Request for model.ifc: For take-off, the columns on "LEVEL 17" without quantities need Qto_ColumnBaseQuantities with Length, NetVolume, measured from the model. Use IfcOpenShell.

First a look at what the model holds.

```python
import ifcopenshell
import ifcopenshell.util.element
import ifcopenshell.util.unit

model = ifcopenshell.open("model.ifc")
print(model.schema)
for unit_type in ("LENGTHUNIT", "AREAUNIT", "VOLUMEUNIT"):
    print(unit_type, ifcopenshell.util.unit.calculate_unit_scale(model, unit_type))
storey = next(s for s in model.by_type("IfcBuildingStorey") if s.Name == "LEVEL 17")
columns = [e for e in ifcopenshell.util.element.get_decomposition(storey) if e.is_a("IfcColumn")]
for e in sorted(columns, key=lambda e: e.id()):
    print(e.id(), e.is_a(), e.Name, list(ifcopenshell.util.element.get_psets(e, qtos_only=True)), sep=" | ")
```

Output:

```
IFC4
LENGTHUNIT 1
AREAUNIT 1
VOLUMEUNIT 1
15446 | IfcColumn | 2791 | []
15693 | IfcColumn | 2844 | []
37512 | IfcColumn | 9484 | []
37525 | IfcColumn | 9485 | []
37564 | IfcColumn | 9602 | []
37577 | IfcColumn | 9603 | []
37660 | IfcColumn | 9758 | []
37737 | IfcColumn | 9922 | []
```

```python
import ifcopenshell
import ifcopenshell.api.pset
import ifcopenshell.geom
import ifcopenshell.util.element
import ifcopenshell.util.shape
import ifcopenshell.util.unit

model = ifcopenshell.open("model.ifc")
unit_scale = ifcopenshell.util.unit.calculate_unit_scale(model)
volume_scale = ifcopenshell.util.unit.calculate_unit_scale(model, "VOLUMEUNIT")
settings = ifcopenshell.geom.settings()

storey = next(s for s in model.by_type("IfcBuildingStorey") if s.Name == "LEVEL 17")
columns = [e for e in ifcopenshell.util.element.get_decomposition(storey) if e.is_a("IfcColumn")]

for e in sorted(columns, key=lambda e: e.id()):
    if ifcopenshell.util.element.get_psets(e, qtos_only=True, should_inherit=False):
        continue
    # Geometry comes back in metres, in the element's own axes.
    shape = ifcopenshell.geom.create_shape(settings, e)
    values = {
        "Length": ifcopenshell.util.shape.get_z(shape.geometry) / unit_scale,
        "NetVolume": ifcopenshell.util.shape.get_volume(shape.geometry) / volume_scale,
    }
    qto = ifcopenshell.api.pset.add_qto(model, product=e, name="Qto_ColumnBaseQuantities")
    ifcopenshell.api.pset.edit_qto(model, qto=qto, properties=values)
    print(e.id(), {k: round(v, 3) for k, v in values.items()})

model.write("model_v2.ifc")
```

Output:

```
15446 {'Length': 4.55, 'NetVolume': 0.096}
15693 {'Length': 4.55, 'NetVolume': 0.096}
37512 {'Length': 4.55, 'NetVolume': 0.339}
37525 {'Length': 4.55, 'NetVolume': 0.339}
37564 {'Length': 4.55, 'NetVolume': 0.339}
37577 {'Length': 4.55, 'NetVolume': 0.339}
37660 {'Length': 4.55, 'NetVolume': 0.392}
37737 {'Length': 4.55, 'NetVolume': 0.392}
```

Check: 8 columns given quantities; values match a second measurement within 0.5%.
